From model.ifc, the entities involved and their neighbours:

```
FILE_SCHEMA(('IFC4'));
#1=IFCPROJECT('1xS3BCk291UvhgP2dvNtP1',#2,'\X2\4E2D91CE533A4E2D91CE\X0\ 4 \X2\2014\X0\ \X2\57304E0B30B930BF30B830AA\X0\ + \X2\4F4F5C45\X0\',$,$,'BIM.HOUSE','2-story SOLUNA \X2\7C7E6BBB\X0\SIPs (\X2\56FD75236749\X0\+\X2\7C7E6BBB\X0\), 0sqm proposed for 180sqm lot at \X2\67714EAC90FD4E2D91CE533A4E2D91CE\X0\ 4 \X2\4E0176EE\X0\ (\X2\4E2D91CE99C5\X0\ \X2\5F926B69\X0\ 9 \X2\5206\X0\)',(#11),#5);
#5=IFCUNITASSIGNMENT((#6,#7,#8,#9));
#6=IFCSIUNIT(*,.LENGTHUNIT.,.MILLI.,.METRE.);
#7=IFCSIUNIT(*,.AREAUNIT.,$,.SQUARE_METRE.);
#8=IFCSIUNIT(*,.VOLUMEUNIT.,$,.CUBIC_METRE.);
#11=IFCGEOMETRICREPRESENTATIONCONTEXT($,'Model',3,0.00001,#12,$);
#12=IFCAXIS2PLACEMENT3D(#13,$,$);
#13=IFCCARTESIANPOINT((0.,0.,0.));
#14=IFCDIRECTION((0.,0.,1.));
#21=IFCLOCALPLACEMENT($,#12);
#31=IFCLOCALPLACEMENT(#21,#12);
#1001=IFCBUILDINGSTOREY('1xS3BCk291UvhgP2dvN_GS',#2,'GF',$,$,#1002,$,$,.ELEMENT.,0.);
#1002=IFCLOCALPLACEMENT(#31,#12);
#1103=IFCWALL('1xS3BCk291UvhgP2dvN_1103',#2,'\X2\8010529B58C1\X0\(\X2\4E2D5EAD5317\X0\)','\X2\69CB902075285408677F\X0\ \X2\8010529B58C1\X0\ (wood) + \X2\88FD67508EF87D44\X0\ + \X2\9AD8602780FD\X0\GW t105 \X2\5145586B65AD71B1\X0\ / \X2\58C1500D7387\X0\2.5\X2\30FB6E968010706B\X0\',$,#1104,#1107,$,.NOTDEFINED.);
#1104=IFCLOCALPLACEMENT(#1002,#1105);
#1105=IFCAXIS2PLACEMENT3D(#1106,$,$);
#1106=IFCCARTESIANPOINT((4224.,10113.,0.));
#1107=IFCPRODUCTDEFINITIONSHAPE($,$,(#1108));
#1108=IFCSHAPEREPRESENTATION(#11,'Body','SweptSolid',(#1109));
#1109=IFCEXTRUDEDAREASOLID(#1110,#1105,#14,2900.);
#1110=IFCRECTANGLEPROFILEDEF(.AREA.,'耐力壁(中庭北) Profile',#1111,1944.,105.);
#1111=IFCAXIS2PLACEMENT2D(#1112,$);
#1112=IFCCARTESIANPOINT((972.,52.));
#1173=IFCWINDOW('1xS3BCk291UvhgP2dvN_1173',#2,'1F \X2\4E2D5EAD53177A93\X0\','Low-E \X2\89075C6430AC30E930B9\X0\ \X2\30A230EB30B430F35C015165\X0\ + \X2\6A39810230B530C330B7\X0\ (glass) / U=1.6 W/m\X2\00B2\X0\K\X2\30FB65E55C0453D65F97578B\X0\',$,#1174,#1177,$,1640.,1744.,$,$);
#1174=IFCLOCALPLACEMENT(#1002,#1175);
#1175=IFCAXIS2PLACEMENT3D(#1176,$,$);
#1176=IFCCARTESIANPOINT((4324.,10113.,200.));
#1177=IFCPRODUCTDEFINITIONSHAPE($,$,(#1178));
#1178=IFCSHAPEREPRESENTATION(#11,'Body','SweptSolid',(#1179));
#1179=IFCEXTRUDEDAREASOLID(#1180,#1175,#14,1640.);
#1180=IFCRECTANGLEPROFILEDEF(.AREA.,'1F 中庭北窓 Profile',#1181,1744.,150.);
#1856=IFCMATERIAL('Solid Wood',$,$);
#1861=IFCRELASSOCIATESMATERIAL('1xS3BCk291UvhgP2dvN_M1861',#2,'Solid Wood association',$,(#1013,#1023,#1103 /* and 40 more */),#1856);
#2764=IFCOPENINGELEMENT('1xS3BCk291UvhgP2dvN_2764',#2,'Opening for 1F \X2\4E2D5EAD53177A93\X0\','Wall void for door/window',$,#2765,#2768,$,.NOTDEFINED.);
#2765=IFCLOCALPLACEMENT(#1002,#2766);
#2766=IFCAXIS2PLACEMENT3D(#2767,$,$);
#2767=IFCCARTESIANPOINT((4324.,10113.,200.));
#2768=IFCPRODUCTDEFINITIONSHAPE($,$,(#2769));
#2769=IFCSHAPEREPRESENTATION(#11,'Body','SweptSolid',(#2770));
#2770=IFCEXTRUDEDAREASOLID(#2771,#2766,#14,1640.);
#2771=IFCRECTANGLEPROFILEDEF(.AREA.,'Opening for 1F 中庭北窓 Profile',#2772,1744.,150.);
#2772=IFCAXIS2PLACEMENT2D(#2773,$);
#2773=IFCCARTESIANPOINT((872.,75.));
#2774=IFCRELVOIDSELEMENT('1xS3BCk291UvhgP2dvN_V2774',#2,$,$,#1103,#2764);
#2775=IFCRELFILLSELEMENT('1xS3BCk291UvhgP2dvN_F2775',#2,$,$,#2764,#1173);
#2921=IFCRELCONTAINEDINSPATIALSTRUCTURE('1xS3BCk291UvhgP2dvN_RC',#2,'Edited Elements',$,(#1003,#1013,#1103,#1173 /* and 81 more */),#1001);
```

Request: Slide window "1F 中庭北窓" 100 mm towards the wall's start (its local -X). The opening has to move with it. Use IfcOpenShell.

```python
import ifcopenshell
import ifcopenshell.api.geometry
import ifcopenshell.util.placement
import ifcopenshell.util.unit

model = ifcopenshell.open("model.ifc")
unit_scale = ifcopenshell.util.unit.calculate_unit_scale(model)

window = model.by_guid("1xS3BCk291UvhgP2dvN_1173")
opening = window.FillsVoids[0].RelatingOpeningElement
wall = opening.VoidsElements[0].RelatingBuildingElement

wall_matrix = ifcopenshell.util.placement.get_local_placement(wall.ObjectPlacement)
shift = wall_matrix[:3, 0] * -0.1 / unit_scale
before = ifcopenshell.util.placement.get_local_placement(window.ObjectPlacement)[:3, 3].copy()

# The window is not placed relative to its opening, so move both.
for product in (opening, window):
    matrix = ifcopenshell.util.placement.get_local_placement(product.ObjectPlacement)
    matrix[:3, 3] += shift
    ifcopenshell.api.geometry.edit_object_placement(model, product=product, matrix=matrix, is_si=False)

after = ifcopenshell.util.placement.get_local_placement(window.ObjectPlacement)[:3, 3]
print("window moved by", (after - before).round(3) + 0.0)

model.write("model_edited.ifc")
```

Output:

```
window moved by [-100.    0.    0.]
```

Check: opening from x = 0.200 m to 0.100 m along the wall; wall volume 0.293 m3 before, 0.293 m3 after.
